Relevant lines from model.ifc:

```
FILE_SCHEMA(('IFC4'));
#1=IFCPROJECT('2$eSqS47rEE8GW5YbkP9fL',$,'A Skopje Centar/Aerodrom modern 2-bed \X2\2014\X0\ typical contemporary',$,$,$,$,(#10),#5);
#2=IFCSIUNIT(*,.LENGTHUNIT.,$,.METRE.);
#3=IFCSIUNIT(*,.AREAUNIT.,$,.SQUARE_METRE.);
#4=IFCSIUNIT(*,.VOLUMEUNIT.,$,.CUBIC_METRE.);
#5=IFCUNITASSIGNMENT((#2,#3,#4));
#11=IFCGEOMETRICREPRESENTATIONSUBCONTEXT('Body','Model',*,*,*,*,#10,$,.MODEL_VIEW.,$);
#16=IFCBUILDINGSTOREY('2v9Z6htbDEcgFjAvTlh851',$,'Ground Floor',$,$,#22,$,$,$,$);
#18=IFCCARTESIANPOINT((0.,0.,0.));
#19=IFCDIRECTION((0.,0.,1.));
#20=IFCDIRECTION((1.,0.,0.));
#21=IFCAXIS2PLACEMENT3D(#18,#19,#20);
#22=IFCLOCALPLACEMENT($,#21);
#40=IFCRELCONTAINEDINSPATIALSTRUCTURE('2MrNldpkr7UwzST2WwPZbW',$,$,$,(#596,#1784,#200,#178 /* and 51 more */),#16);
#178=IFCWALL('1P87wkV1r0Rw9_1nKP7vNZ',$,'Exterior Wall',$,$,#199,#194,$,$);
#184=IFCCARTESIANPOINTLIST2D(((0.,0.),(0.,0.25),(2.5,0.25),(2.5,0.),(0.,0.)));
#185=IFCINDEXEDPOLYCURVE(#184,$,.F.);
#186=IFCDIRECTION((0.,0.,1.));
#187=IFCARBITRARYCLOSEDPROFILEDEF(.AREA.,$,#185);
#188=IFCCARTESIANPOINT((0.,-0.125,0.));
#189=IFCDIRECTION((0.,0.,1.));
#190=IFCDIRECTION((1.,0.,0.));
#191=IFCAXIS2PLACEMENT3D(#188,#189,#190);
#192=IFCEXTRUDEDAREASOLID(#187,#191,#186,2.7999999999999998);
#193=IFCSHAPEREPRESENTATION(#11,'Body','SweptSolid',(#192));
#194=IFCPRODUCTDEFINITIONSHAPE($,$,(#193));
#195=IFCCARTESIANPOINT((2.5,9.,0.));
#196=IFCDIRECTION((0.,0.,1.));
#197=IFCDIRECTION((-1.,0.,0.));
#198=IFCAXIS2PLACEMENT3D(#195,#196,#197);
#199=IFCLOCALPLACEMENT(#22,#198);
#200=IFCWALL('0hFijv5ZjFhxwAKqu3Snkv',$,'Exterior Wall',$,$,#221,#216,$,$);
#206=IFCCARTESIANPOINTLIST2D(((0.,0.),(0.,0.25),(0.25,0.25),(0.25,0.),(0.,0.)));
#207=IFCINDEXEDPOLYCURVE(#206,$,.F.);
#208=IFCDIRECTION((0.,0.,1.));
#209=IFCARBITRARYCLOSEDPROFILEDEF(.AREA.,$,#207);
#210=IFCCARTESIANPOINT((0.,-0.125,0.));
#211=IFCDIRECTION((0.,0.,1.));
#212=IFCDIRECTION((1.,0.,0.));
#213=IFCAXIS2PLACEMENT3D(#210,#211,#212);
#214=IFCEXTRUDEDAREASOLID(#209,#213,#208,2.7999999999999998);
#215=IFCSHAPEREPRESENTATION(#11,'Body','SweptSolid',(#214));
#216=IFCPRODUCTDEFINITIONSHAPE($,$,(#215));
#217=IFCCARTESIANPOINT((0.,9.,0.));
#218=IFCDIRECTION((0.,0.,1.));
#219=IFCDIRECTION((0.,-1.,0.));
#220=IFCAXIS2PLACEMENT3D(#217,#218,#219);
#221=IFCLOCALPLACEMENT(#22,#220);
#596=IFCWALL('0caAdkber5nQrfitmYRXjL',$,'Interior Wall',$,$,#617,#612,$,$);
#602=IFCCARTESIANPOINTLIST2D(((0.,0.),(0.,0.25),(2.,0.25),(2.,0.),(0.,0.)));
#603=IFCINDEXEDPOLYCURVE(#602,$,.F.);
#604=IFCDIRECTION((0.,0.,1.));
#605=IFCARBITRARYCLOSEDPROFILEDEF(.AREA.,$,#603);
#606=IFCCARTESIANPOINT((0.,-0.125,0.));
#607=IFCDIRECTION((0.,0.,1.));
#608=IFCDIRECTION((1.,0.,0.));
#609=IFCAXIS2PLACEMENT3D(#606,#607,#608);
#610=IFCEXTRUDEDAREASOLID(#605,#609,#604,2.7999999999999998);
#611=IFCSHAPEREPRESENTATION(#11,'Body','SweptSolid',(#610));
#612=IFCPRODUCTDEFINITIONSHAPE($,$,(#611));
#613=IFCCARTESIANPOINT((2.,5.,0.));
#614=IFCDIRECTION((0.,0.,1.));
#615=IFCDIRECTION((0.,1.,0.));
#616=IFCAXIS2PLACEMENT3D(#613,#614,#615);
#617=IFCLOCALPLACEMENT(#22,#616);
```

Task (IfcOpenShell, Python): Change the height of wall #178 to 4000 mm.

```python
import ifcopenshell
import ifcopenshell.geom
import ifcopenshell.util.representation
import ifcopenshell.util.shape

model = ifcopenshell.open("model.ifc")
settings = ifcopenshell.geom.settings()


def volume(element):
    """Net volume in cubic metres, openings subtracted."""
    shape = ifcopenshell.geom.create_shape(settings, element)
    return ifcopenshell.util.shape.get_volume(shape.geometry)


wall = model.by_guid("1P87wkV1r0Rw9_1nKP7vNZ")
before = volume(wall)

body = ifcopenshell.util.representation.get_representation(wall, "Model", "Body")
solid = body.Items[0]
old_height = solid.Depth
solid.Depth = 4.0
after = volume(wall)

print(f"height {old_height:g} -> {solid.Depth:g}, volume {before:.3f} -> {after:.3f} m3")

model.write("model_v2.ifc")
```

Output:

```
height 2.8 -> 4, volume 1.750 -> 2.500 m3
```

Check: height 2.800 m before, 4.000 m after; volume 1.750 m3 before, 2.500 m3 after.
